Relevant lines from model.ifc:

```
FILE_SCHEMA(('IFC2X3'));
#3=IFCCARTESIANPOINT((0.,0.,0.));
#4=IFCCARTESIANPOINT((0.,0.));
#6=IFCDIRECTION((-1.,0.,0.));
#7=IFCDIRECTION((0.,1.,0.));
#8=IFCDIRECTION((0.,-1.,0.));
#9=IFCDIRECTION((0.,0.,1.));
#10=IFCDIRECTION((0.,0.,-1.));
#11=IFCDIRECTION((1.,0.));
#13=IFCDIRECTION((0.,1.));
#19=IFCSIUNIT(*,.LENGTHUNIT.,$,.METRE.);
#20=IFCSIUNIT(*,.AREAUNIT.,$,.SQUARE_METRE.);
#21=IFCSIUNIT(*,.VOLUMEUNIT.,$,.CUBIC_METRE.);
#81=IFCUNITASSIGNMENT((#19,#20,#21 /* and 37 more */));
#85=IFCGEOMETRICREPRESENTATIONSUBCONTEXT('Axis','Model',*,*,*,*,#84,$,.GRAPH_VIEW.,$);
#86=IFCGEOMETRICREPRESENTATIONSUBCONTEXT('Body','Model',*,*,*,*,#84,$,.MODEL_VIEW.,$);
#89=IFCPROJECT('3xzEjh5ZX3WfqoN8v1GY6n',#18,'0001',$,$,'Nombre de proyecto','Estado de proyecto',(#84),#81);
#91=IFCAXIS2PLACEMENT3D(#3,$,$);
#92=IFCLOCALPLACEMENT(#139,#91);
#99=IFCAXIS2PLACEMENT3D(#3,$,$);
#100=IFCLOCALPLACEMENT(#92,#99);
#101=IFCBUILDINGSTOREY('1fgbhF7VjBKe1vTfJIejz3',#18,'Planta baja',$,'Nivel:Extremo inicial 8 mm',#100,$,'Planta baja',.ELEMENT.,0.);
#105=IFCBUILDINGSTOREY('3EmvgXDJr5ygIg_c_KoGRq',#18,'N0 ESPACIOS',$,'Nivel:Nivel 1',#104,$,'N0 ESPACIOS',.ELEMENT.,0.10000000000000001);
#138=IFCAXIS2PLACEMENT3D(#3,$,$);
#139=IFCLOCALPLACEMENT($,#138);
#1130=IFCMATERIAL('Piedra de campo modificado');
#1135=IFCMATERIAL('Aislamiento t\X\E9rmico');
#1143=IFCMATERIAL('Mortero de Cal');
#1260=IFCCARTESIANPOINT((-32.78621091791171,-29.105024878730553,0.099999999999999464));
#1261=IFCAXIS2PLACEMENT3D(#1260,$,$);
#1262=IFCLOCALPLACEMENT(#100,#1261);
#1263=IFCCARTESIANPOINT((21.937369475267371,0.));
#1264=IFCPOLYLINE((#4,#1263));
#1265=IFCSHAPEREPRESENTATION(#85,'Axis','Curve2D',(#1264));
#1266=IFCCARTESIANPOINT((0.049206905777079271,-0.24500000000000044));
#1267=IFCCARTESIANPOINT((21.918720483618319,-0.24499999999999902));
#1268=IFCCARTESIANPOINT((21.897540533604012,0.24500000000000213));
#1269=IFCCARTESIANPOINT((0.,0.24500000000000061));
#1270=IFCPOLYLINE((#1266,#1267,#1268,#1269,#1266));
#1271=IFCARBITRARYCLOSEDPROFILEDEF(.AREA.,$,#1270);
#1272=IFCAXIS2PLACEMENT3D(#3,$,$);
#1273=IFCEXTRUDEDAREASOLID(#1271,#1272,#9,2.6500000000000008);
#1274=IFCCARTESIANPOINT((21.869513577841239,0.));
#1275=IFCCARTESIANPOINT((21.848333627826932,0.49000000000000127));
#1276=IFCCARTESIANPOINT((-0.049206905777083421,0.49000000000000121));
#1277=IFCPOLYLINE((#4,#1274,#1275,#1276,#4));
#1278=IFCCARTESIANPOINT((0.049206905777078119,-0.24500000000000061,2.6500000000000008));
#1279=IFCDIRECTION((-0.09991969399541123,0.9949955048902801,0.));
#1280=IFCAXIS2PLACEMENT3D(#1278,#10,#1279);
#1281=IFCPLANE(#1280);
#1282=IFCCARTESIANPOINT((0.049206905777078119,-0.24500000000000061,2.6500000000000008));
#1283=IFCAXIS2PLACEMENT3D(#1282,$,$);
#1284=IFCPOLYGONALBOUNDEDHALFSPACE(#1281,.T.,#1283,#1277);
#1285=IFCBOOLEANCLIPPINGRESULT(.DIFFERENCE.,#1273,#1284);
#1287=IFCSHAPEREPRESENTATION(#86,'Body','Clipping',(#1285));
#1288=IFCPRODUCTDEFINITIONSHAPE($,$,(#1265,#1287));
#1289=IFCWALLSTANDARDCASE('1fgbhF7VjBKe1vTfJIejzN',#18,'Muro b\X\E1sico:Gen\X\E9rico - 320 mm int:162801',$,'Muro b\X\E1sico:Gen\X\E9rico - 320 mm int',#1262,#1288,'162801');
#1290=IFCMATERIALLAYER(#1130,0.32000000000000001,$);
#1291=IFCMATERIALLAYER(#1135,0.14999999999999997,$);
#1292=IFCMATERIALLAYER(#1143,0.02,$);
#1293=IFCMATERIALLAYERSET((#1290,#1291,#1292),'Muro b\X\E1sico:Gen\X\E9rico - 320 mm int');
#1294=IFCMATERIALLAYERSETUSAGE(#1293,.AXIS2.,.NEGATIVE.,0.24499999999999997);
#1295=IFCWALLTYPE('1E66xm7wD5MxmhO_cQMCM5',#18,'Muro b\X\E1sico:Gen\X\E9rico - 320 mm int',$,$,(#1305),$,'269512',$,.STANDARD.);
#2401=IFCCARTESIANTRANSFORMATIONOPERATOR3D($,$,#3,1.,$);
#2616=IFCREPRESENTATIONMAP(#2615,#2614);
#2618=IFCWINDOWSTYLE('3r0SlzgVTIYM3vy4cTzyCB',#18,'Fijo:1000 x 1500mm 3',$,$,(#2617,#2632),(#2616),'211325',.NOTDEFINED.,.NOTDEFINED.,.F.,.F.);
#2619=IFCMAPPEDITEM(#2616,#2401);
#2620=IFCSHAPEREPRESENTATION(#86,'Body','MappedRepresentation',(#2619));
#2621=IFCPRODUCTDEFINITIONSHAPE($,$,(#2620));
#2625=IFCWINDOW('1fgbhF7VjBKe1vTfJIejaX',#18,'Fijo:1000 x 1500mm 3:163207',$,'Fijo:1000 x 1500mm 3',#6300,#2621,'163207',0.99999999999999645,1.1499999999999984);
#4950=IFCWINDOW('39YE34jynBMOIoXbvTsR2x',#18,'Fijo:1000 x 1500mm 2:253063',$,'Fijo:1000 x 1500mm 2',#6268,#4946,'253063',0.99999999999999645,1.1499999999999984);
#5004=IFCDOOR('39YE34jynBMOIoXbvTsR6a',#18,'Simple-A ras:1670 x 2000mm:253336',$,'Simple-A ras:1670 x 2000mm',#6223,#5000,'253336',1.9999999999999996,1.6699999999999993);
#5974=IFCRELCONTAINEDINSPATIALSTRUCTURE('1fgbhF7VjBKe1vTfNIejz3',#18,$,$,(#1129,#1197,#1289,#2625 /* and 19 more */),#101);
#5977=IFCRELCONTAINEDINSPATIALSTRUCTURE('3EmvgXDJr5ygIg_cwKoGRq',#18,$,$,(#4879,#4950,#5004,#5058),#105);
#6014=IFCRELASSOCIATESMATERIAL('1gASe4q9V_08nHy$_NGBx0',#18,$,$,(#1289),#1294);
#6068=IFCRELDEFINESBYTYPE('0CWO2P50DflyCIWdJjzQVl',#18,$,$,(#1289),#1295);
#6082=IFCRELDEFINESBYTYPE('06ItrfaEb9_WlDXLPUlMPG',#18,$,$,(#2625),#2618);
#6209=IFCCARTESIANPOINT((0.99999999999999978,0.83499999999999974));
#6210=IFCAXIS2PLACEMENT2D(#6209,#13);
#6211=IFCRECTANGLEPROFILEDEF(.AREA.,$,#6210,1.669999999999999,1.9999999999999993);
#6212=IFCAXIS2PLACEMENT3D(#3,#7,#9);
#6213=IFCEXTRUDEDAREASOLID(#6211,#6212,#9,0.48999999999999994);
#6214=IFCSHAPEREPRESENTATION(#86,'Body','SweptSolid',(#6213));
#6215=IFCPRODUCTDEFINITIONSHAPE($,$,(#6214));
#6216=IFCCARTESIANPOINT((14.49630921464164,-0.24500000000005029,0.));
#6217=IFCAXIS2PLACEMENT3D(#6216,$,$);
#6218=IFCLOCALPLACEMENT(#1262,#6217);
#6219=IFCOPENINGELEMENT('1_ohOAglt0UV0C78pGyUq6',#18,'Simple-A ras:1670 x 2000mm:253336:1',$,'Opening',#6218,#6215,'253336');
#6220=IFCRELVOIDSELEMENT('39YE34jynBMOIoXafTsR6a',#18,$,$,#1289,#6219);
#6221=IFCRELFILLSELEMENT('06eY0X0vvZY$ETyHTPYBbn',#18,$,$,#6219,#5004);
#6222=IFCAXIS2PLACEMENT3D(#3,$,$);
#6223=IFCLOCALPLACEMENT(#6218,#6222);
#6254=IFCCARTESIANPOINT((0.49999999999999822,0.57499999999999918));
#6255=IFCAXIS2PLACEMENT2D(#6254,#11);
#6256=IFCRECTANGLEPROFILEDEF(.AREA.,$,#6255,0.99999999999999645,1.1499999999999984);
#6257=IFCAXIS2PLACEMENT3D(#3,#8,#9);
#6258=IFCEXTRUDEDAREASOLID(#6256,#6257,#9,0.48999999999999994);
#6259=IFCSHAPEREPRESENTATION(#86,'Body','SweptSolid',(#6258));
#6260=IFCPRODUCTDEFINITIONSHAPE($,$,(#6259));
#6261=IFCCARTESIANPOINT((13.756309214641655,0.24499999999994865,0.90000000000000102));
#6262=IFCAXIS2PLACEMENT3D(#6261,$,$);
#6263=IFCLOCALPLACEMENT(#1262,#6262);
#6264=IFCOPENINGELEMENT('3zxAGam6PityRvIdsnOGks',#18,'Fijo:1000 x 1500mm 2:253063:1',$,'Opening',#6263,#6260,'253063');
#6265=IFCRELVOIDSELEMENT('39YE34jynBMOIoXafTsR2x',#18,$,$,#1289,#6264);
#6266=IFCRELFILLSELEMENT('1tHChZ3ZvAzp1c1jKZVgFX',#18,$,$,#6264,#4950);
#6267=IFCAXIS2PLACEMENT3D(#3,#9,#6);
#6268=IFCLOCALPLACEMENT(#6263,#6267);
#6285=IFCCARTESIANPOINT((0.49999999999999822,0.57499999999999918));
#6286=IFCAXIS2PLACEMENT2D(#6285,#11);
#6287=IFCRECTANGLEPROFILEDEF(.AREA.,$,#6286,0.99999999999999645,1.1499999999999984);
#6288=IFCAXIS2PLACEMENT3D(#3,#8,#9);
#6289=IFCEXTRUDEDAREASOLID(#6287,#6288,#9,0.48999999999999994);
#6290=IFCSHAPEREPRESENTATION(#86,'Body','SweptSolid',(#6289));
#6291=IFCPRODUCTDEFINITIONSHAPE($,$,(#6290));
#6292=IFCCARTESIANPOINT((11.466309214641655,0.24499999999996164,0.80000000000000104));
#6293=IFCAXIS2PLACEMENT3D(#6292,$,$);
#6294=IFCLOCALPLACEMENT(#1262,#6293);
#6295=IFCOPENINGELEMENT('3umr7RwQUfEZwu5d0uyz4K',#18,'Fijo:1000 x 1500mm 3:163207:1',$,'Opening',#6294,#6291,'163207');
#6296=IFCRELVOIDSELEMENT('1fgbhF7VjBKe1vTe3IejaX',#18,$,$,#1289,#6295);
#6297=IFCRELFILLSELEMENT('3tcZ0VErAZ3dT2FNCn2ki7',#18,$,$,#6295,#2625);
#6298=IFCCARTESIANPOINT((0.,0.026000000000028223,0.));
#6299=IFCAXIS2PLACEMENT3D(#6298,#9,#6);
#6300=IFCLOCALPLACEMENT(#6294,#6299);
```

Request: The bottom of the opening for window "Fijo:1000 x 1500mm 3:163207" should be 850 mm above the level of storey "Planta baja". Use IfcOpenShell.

```python
import numpy as np
import ifcopenshell
import ifcopenshell.api.geometry
import ifcopenshell.geom
import ifcopenshell.util.element
import ifcopenshell.util.placement
import ifcopenshell.util.shape
import ifcopenshell.util.unit

model = ifcopenshell.open("model.ifc")
unit_scale = ifcopenshell.util.unit.calculate_unit_scale(model)

window = model.by_id(2625)
opening = window.FillsVoids[0].RelatingOpeningElement
storey = ifcopenshell.util.element.get_container(window, ifc_class="IfcBuildingStorey")
level = ifcopenshell.util.placement.get_local_placement(storey.ObjectPlacement)[2, 3]

# The opening's origin need not be at the sill, so measure its lowest point.
shape = ifcopenshell.geom.create_shape(ifcopenshell.geom.settings(), opening)
bottom = ifcopenshell.util.shape.get_shape_bottom_elevation(shape, shape.geometry) / unit_scale
dz = level + 0.85 / unit_scale - bottom

shift = np.array([0.0, 0.0, dz])
# The window is placed relative to its opening, so it follows when the opening moves.
matrix = ifcopenshell.util.placement.get_local_placement(opening.ObjectPlacement)
matrix[:3, 3] += shift
ifcopenshell.api.geometry.edit_object_placement(
    model, product=opening, matrix=matrix, is_si=False, should_transform_children=True
)

print(f"moved by {dz * unit_scale:+.3f} m")

model.write("model_v2.ifc")
```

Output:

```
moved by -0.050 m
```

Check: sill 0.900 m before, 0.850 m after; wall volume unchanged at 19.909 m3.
